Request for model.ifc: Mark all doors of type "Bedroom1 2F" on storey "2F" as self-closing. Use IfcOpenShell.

First a look at what the model holds.

```python
import ifcopenshell
import ifcopenshell.util.element

model = ifcopenshell.open("model.ifc")
print(model.schema)
storey = next(s for s in model.by_type("IfcBuildingStorey") if s.Name == "2F")
doors = [e for e in ifcopenshell.util.element.get_decomposition(storey) if e.is_a("IfcDoor")]
seen = {}
for e in doors:
    element_type = ifcopenshell.util.element.get_type(e)
    key = (element_type.Name if element_type != e and element_type else None, ifcopenshell.util.element.get_pset(e, "Pset_DoorCommon", "SelfClosing"))
    seen[key] = seen.get(key, 0) + 1
for (name, value), count in sorted(seen.items(), key=str):
    print(count, "x", name, "|", value)
```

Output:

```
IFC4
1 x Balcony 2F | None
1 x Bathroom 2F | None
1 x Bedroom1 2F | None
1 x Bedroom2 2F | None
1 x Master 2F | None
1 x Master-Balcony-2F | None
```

```python
import ifcopenshell
import ifcopenshell.api.pset
import ifcopenshell.util.element

model = ifcopenshell.open("model.ifc")

storey = next(s for s in model.by_type("IfcBuildingStorey") if s.Name == "2F")
doors = [e for e in ifcopenshell.util.element.get_decomposition(storey) if e.is_a("IfcDoor")]

count = 0
for e in doors:
    element_type = ifcopenshell.util.element.get_type(e)
    if element_type in (None, e) or element_type.Name != "Bedroom1 2F":
        continue
    # add_pset returns the element's existing set when there is one.
    pset = ifcopenshell.api.pset.add_pset(model, product=e, name="Pset_DoorCommon")
    ifcopenshell.api.pset.edit_pset(model, pset=pset, properties={"SelfClosing": True})
    count += 1

print(count, "doors updated")

model.write("model_v2.ifc")
```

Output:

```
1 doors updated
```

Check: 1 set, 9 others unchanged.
